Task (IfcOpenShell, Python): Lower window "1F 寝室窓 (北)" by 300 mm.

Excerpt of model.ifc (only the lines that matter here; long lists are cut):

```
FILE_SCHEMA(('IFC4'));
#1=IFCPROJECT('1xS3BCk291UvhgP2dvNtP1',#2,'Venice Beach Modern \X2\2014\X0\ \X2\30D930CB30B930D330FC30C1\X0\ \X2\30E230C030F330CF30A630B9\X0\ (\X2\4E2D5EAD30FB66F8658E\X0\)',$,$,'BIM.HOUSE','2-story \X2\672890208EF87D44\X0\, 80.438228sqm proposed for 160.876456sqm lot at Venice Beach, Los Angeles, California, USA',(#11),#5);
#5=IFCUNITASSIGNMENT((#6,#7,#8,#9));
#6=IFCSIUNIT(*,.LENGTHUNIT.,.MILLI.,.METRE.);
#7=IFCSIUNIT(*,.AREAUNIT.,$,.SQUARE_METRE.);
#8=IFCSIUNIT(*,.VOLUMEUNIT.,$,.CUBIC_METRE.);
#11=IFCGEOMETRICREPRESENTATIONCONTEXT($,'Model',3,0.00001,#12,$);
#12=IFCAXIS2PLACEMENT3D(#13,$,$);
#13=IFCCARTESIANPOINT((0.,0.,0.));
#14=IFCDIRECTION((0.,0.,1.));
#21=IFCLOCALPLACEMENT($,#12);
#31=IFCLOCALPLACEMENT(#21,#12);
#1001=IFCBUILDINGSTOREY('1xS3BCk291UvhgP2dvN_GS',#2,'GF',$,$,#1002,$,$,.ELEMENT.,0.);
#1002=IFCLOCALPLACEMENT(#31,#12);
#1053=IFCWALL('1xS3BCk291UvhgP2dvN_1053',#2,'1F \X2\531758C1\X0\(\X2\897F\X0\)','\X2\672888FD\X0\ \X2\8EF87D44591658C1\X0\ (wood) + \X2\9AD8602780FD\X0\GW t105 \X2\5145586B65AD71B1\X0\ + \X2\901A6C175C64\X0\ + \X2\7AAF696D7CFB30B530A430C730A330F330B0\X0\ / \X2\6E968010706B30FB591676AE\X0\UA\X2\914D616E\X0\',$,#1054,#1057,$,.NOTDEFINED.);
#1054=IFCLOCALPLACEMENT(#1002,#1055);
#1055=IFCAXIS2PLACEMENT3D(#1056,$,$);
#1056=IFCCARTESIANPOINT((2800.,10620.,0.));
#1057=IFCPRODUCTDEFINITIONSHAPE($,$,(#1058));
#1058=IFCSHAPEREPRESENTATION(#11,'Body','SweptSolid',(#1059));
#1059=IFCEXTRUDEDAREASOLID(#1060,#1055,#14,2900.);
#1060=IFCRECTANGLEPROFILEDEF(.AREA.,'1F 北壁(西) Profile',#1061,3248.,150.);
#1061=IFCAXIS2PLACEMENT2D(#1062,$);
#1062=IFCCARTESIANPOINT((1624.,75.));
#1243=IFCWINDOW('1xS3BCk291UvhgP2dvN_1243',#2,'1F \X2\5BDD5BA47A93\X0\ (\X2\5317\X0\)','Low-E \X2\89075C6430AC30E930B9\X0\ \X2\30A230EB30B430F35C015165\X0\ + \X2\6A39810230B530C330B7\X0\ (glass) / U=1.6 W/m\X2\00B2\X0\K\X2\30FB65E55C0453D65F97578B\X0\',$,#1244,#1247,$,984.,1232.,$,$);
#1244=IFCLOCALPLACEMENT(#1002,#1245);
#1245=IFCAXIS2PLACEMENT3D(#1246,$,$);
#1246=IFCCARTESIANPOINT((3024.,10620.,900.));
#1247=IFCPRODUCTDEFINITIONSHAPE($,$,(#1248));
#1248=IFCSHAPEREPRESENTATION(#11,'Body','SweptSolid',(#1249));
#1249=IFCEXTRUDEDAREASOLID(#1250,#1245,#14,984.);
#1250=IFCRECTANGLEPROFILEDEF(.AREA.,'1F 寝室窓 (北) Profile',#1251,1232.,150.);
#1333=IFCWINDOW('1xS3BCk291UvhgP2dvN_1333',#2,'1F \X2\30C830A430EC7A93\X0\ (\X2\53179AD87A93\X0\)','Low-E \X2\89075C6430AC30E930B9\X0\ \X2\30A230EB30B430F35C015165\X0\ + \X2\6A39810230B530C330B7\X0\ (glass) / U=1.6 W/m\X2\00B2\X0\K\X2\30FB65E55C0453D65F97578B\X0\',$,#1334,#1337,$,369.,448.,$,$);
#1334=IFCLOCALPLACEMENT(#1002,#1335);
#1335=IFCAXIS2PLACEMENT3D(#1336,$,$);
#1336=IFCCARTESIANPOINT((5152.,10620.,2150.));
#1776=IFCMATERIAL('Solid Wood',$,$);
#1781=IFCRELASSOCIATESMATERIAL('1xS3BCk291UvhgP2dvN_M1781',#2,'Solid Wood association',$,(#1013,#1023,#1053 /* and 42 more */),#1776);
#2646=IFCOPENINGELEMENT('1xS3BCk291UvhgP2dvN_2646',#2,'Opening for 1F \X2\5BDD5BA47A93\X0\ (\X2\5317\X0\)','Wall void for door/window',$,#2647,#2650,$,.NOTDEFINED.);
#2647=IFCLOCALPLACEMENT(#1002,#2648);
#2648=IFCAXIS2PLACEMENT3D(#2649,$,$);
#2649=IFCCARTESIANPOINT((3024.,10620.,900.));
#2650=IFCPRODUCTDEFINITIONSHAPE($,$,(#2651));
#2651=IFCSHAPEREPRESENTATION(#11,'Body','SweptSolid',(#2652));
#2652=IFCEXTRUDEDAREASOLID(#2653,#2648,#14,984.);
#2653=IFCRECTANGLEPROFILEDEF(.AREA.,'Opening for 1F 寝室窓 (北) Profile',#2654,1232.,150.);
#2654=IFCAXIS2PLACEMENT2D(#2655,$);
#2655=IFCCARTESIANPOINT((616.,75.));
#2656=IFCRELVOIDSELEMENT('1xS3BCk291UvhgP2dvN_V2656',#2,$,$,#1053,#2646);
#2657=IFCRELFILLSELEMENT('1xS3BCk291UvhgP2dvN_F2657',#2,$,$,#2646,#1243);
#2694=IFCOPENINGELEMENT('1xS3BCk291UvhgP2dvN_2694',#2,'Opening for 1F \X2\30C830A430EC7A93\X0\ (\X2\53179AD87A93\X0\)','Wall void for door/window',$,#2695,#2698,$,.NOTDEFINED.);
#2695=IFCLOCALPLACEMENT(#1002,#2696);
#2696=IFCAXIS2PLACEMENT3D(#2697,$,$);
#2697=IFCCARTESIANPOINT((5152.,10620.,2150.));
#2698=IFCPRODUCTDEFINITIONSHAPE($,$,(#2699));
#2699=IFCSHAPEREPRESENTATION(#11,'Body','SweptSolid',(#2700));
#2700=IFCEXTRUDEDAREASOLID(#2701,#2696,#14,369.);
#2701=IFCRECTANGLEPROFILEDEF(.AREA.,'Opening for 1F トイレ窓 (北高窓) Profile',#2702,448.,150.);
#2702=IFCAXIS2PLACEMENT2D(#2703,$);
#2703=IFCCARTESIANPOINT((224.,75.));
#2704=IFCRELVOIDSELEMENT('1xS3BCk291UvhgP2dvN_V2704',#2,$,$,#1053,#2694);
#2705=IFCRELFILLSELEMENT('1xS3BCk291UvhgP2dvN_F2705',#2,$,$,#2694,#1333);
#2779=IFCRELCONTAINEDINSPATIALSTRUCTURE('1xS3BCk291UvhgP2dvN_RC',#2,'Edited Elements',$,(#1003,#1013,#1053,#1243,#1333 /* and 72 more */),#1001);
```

```python
import numpy as np
import ifcopenshell
import ifcopenshell.api.geometry
import ifcopenshell.util.placement
import ifcopenshell.util.unit

model = ifcopenshell.open("model.ifc")
unit_scale = ifcopenshell.util.unit.calculate_unit_scale(model)

window = model.by_guid("1xS3BCk291UvhgP2dvN_1243")
opening = window.FillsVoids[0].RelatingOpeningElement
dz = -300.0

shift = np.array([0.0, 0.0, dz])
# The window is not placed relative to its opening, so move both.
for product in (opening, window):
    matrix = ifcopenshell.util.placement.get_local_placement(product.ObjectPlacement)
    matrix[:3, 3] += shift
    ifcopenshell.api.geometry.edit_object_placement(model, product=product, matrix=matrix, is_si=False)

print(f"moved by {dz * unit_scale:+.3f} m")

model.write("model_rev.ifc")
```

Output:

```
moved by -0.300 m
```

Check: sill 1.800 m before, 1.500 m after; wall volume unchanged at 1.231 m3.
